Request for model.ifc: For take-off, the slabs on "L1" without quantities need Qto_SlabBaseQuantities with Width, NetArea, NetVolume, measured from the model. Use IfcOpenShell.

First a look at what the model holds.

```python
import ifcopenshell
import ifcopenshell.util.element
import ifcopenshell.util.unit

model = ifcopenshell.open("model.ifc")
print(model.schema)
for unit_type in ("LENGTHUNIT", "AREAUNIT", "VOLUMEUNIT"):
    print(unit_type, ifcopenshell.util.unit.calculate_unit_scale(model, unit_type))
storey = next(s for s in model.by_type("IfcBuildingStorey") if s.Name == "L1")
slabs = [e for e in ifcopenshell.util.element.get_decomposition(storey) if e.is_a("IfcSlab")]
for e in sorted(slabs, key=lambda e: e.id()):
    print(e.id(), e.is_a(), e.Name, list(ifcopenshell.util.element.get_psets(e, qtos_only=True)), sep=" | ")
```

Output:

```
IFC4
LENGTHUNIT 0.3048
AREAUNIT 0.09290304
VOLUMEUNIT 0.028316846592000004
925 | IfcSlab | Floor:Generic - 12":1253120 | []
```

```python
import ifcopenshell
import ifcopenshell.api.pset
import ifcopenshell.geom
import ifcopenshell.util.element
import ifcopenshell.util.shape
import ifcopenshell.util.unit

model = ifcopenshell.open("model.ifc")
unit_scale = ifcopenshell.util.unit.calculate_unit_scale(model)
area_scale = ifcopenshell.util.unit.calculate_unit_scale(model, "AREAUNIT")
volume_scale = ifcopenshell.util.unit.calculate_unit_scale(model, "VOLUMEUNIT")
settings = ifcopenshell.geom.settings()

storey = next(s for s in model.by_type("IfcBuildingStorey") if s.Name == "L1")
slabs = [e for e in ifcopenshell.util.element.get_decomposition(storey) if e.is_a("IfcSlab")]

for e in sorted(slabs, key=lambda e: e.id()):
    if ifcopenshell.util.element.get_psets(e, qtos_only=True, should_inherit=False):
        continue
    # Geometry comes back in metres, in the element's own axes.
    shape = ifcopenshell.geom.create_shape(settings, e)
    values = {
        "Width": ifcopenshell.util.shape.get_z(shape.geometry) / unit_scale,
        "NetArea": ifcopenshell.util.shape.get_footprint_area(shape.geometry) / area_scale,
        "NetVolume": ifcopenshell.util.shape.get_volume(shape.geometry) / volume_scale,
    }
    qto = ifcopenshell.api.pset.add_qto(model, product=e, name="Qto_SlabBaseQuantities")
    ifcopenshell.api.pset.edit_qto(model, qto=qto, properties=values)
    print(e.id(), {k: round(v, 3) for k, v in values.items()})

model.write("model_v2.ifc")
```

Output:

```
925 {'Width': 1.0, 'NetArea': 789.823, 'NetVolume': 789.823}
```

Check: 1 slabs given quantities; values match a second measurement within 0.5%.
